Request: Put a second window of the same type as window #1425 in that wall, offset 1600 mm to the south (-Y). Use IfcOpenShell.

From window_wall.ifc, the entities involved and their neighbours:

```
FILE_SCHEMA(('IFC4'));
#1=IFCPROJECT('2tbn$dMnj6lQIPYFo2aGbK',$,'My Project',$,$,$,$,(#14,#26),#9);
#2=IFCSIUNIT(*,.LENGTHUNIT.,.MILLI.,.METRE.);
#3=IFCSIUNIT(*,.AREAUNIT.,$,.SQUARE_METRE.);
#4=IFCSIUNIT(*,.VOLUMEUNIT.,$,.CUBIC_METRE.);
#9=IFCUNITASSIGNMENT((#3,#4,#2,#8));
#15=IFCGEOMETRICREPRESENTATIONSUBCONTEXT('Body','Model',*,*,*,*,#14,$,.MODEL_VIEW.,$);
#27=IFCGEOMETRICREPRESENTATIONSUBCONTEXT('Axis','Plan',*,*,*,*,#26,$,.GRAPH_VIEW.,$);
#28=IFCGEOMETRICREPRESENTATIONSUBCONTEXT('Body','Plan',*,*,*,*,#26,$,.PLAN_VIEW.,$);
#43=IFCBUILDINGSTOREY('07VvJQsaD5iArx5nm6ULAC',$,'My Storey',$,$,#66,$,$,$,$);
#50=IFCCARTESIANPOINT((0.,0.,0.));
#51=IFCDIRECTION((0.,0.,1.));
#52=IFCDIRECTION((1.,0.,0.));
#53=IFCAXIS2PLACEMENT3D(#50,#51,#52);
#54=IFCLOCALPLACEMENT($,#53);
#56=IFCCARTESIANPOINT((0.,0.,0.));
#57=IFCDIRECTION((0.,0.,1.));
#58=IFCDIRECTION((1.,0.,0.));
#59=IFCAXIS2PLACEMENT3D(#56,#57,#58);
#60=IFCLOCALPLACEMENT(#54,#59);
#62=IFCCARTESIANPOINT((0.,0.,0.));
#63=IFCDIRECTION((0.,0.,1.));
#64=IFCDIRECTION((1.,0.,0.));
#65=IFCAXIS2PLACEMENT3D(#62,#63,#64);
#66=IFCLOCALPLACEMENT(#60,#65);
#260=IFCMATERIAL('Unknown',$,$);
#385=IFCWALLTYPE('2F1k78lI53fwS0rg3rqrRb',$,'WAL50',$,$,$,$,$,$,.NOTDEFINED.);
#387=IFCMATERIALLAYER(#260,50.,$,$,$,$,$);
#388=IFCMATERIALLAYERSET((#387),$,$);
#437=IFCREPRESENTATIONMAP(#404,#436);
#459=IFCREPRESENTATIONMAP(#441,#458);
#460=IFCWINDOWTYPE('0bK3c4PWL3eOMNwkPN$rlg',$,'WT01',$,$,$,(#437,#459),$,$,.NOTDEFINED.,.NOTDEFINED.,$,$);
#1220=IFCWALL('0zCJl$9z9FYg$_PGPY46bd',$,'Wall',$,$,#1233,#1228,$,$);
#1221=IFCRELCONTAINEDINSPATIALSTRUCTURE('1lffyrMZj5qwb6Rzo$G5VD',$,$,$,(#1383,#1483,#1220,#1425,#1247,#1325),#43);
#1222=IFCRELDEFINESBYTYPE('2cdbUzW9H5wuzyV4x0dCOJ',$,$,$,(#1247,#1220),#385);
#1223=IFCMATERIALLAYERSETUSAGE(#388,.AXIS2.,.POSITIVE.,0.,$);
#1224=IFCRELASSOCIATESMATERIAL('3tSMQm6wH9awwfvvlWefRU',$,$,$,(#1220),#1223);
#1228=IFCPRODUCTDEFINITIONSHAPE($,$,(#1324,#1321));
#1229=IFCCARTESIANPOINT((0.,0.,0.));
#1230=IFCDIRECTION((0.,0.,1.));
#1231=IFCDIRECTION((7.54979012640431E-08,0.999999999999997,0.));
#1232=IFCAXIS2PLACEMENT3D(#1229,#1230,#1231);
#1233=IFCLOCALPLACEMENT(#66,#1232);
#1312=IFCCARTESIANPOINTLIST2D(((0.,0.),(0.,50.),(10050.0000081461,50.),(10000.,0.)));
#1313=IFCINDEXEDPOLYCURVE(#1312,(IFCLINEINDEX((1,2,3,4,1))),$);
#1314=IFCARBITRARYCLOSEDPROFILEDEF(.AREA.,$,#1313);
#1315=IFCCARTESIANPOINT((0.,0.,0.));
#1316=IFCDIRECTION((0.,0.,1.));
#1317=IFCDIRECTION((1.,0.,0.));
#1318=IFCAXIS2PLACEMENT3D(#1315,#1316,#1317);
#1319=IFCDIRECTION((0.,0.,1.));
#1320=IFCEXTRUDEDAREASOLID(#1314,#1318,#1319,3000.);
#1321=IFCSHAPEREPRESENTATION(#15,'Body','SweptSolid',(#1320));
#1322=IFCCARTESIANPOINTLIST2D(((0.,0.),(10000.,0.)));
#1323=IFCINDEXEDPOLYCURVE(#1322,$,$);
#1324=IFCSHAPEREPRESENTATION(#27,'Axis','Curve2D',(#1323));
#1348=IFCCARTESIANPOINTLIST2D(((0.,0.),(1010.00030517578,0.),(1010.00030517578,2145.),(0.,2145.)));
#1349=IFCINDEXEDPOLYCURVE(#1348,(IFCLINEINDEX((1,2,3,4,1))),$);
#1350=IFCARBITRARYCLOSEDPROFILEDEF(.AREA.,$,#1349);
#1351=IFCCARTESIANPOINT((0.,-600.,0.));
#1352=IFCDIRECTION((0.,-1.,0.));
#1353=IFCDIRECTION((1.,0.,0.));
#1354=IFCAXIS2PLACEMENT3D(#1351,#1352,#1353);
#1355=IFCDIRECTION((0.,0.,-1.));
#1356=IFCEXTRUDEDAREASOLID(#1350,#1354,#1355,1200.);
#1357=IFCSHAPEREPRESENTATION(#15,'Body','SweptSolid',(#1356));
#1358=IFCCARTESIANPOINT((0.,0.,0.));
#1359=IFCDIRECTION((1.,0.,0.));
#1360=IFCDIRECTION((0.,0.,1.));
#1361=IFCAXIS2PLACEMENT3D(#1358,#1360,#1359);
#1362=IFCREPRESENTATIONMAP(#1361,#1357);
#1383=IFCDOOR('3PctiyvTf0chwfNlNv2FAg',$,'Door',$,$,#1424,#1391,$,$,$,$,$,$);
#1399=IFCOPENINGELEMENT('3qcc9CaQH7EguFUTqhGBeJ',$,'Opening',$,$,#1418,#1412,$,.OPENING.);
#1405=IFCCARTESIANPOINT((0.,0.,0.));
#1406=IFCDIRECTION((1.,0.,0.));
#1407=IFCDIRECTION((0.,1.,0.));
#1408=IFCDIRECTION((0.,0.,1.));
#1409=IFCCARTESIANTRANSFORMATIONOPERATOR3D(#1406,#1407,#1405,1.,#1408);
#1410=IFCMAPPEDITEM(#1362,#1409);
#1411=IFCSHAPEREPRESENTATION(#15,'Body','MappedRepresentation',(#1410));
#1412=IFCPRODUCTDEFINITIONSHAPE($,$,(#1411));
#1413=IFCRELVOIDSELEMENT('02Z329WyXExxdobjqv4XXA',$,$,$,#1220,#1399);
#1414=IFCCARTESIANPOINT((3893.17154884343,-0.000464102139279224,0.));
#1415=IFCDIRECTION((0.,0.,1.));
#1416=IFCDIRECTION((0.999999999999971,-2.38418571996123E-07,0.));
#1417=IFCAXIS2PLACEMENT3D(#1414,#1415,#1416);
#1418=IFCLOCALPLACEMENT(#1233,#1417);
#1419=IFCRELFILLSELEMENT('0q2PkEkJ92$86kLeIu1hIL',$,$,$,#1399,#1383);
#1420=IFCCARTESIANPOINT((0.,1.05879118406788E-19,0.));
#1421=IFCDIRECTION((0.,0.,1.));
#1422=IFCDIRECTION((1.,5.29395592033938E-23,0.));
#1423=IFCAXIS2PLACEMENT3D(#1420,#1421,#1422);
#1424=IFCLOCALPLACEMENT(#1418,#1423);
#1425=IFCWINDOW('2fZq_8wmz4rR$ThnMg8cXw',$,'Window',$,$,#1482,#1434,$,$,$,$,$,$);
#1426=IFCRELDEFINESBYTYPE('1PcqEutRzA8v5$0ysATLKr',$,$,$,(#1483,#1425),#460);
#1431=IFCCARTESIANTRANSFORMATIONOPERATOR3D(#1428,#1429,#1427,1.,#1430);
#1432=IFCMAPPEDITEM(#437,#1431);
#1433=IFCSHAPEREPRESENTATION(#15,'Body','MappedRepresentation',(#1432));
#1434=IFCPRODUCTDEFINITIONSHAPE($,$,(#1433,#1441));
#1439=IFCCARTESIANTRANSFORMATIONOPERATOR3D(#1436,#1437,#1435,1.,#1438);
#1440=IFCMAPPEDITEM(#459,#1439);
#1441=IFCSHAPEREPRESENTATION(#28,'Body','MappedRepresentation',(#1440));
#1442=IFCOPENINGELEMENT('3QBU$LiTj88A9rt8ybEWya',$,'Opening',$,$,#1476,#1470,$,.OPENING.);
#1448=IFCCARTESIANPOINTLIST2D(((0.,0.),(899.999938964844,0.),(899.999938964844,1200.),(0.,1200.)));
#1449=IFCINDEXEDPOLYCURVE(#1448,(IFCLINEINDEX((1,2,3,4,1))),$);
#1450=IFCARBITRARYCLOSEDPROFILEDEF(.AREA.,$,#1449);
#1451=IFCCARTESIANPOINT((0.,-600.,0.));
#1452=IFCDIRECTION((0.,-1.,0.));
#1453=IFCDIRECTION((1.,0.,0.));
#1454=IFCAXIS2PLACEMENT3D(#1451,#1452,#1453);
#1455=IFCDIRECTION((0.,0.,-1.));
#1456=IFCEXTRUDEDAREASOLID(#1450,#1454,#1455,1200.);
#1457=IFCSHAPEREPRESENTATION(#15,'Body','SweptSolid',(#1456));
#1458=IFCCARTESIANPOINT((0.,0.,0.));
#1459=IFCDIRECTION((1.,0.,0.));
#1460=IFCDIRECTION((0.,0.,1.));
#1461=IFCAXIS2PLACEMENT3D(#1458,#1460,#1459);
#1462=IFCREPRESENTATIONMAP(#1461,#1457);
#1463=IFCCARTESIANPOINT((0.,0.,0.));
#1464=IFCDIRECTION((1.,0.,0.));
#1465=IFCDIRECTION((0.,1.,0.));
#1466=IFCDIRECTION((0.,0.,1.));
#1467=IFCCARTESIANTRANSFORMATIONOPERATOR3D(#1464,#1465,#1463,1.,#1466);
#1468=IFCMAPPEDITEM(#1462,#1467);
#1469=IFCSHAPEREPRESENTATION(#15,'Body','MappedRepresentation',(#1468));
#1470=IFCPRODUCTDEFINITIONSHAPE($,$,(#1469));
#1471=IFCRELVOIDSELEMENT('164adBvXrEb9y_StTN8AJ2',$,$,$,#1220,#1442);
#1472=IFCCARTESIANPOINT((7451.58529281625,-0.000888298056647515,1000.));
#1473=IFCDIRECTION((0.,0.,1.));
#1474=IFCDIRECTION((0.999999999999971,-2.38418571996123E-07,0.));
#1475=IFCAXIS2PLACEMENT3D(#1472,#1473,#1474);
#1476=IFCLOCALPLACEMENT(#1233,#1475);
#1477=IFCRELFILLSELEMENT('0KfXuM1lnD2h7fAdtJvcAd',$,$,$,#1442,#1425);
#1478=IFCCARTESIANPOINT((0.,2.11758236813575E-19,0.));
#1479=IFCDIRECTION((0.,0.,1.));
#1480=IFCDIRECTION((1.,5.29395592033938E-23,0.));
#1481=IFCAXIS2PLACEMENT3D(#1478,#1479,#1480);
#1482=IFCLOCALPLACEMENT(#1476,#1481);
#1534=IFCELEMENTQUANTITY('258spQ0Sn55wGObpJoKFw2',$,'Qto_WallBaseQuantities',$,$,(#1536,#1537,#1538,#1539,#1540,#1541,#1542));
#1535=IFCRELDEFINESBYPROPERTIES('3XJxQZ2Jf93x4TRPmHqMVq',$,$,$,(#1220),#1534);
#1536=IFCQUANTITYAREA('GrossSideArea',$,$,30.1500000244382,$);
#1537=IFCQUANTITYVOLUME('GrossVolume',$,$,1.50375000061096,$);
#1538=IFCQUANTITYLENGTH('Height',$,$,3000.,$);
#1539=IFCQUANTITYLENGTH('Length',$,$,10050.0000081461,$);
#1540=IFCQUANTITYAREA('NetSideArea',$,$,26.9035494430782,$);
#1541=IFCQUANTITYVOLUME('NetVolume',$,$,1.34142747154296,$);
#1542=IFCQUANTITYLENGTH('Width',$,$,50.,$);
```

```python
import ifcopenshell
import ifcopenshell.api.feature
import ifcopenshell.api.geometry
import ifcopenshell.api.pset
import ifcopenshell.api.root
import ifcopenshell.geom
import ifcopenshell.util.element
import ifcopenshell.util.placement
import ifcopenshell.util.shape
import ifcopenshell.util.unit

model = ifcopenshell.open("window_wall.ifc")
area_scale = ifcopenshell.util.unit.calculate_unit_scale(model, "AREAUNIT")
volume_scale = ifcopenshell.util.unit.calculate_unit_scale(model, "VOLUMEUNIT")
settings = ifcopenshell.geom.settings()


def volume(element):
    """Net volume in cubic metres, openings subtracted."""
    shape = ifcopenshell.geom.create_shape(settings, element)
    return ifcopenshell.util.shape.get_volume(shape.geometry)


window = model.by_guid("2fZq_8wmz4rR$ThnMg8cXw")
opening = window.FillsVoids[0].RelatingOpeningElement
wall = opening.VoidsElements[0].RelatingBuildingElement
before = volume(wall)
shift = ifcopenshell.util.placement.get_local_placement(wall.ObjectPlacement)[:3, 0] * -1600.0

# copy_class copies the void relationship, type, container and properties, but no geometry.
new_opening = ifcopenshell.api.root.copy_class(model, product=opening)
new_opening.Representation = ifcopenshell.util.element.copy_deep(
    model, opening.Representation, exclude=["IfcGeometricRepresentationContext", "IfcRepresentationMap"]
)
new_window = ifcopenshell.api.root.copy_class(model, product=window)
new_window.Representation = ifcopenshell.util.element.copy_deep(
    model, window.Representation, exclude=["IfcGeometricRepresentationContext", "IfcRepresentationMap"]
)
ifcopenshell.api.feature.add_filling(model, opening=new_opening, element=new_window)

for old, new in ((opening, new_opening), (window, new_window)):
    matrix = ifcopenshell.util.placement.get_local_placement(old.ObjectPlacement)
    matrix[:3, 3] += shift
    ifcopenshell.api.geometry.edit_object_placement(model, product=new, matrix=matrix, is_si=False)

after = volume(wall)
thickness = 0.05  # wall thickness in metres

# Update the wall's stored quantities.
qto = model.by_id(ifcopenshell.util.element.get_pset(wall, "Qto_WallBaseQuantities", should_inherit=False)["id"])
ifcopenshell.api.pset.edit_qto(model, qto=qto, properties={
    "NetSideArea": after / thickness / area_scale,
    "NetVolume": after / volume_scale,
})

print(f"wall volume {before:.3f} -> {after:.3f} m3")

model.write("window_wall_v2.ifc")
```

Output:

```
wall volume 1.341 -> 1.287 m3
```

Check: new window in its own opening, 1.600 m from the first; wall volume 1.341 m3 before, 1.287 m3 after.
